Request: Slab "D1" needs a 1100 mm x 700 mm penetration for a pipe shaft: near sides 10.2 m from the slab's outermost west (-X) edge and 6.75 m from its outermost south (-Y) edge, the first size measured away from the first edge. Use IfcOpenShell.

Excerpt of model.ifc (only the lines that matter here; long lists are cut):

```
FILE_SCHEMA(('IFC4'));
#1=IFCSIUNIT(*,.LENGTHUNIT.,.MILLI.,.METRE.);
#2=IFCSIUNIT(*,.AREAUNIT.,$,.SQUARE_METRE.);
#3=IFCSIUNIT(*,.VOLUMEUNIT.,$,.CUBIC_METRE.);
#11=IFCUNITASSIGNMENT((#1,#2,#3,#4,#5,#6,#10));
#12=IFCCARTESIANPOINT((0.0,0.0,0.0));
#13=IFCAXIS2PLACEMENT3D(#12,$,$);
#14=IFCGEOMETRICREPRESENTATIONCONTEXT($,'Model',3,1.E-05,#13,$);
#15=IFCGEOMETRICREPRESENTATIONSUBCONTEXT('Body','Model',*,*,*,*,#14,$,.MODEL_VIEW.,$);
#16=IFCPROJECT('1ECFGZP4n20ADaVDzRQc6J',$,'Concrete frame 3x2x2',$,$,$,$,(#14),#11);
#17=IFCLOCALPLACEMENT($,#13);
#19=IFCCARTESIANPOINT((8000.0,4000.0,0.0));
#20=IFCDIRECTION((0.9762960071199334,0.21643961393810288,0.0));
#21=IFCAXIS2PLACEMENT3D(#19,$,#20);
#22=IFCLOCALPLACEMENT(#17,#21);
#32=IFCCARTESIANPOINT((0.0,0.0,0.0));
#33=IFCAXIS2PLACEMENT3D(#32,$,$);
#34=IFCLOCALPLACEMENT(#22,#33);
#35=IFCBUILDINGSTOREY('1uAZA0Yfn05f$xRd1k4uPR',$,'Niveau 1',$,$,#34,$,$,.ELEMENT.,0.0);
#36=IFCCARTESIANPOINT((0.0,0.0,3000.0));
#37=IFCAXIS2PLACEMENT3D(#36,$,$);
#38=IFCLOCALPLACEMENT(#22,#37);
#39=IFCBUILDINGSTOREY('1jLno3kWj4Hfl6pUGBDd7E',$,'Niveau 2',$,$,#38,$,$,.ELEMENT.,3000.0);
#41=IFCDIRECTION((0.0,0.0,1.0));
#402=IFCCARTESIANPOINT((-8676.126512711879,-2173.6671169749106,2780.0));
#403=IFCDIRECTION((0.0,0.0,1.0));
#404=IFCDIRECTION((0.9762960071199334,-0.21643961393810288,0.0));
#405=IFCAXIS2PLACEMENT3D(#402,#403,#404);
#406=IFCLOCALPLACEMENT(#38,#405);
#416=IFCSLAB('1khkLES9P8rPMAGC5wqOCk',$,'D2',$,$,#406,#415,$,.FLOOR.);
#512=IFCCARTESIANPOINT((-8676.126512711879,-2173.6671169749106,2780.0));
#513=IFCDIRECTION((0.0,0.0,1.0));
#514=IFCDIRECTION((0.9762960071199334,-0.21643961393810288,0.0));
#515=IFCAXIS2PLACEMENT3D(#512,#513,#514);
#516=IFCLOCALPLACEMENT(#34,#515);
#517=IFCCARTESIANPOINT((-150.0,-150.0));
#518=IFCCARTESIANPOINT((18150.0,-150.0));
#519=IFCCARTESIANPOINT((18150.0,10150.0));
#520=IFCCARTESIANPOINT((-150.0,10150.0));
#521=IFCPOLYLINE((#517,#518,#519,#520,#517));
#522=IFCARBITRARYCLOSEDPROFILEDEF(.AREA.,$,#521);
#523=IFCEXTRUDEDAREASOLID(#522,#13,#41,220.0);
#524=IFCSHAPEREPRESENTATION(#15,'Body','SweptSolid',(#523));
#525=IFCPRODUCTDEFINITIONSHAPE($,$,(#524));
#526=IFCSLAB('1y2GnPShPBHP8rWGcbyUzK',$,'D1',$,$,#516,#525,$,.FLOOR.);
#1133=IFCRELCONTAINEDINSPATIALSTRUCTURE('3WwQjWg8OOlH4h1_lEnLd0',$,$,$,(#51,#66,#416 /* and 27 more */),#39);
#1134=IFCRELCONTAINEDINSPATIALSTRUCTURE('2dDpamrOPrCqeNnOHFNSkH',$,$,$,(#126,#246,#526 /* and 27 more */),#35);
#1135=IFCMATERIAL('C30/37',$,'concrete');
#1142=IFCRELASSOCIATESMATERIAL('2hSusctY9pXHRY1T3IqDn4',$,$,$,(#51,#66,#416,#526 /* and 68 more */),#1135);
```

```python
import numpy as np
import ifcopenshell
import ifcopenshell.api.feature
import ifcopenshell.api.geometry
import ifcopenshell.api.root
import ifcopenshell.geom
import ifcopenshell.util.placement
import ifcopenshell.util.representation
import ifcopenshell.util.shape
import ifcopenshell.util.unit

model = ifcopenshell.open("model.ifc")
unit_scale = ifcopenshell.util.unit.calculate_unit_scale(model)
settings = ifcopenshell.geom.settings()


def volume(element):
    """Net volume in cubic metres, openings subtracted."""
    shape = ifcopenshell.geom.create_shape(settings, element)
    return ifcopenshell.util.shape.get_volume(shape.geometry)


slab = model.by_guid("1y2GnPShPBHP8rWGcbyUzK")
before = volume(slab)

# Extent in the slab's own axes, in metres. The edges named are its -X and -Y sides.
slab_shape = ifcopenshell.geom.create_shape(settings, slab)
vertices = ifcopenshell.util.shape.get_vertices(slab_shape.geometry)
x_min, y_min, bottom = vertices.min(axis=0)
top = vertices[:, 2].max()

opening = ifcopenshell.api.root.create_entity(model, ifc_class="IfcOpeningElement", name="Pipe shaft opening", predefined_type="OPENING")
context = ifcopenshell.util.representation.get_context(model, "Model", "Body", "MODEL_VIEW")
width, depth = 1.1, 0.7
outline = [(0.0, 0.0), (width, 0.0), (width, depth), (0.0, depth), (0.0, 0.0)]
# Overshoot both faces by 50 mm so the cut is clean.
shape = ifcopenshell.api.geometry.add_slab_representation(
    model, context=context, depth=top - bottom + 0.1, polyline=outline
)
ifcopenshell.api.geometry.assign_representation(model, product=opening, representation=shape)

matrix = ifcopenshell.util.placement.get_local_placement(slab.ObjectPlacement)
matrix[:, 3] = matrix @ np.append(np.array([x_min + 10.2, y_min + 6.75, bottom - 0.05]) / unit_scale, 1.0)
ifcopenshell.api.geometry.edit_object_placement(model, product=opening, matrix=matrix, is_si=False)
ifcopenshell.api.feature.add_feature(model, feature=opening, element=slab)

after = volume(slab)

print(f"slab volume {before:.3f} -> {after:.3f} m3")

model.write("model_updated.ifc")
```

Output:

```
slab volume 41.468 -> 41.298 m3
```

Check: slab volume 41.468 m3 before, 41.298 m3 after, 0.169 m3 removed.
